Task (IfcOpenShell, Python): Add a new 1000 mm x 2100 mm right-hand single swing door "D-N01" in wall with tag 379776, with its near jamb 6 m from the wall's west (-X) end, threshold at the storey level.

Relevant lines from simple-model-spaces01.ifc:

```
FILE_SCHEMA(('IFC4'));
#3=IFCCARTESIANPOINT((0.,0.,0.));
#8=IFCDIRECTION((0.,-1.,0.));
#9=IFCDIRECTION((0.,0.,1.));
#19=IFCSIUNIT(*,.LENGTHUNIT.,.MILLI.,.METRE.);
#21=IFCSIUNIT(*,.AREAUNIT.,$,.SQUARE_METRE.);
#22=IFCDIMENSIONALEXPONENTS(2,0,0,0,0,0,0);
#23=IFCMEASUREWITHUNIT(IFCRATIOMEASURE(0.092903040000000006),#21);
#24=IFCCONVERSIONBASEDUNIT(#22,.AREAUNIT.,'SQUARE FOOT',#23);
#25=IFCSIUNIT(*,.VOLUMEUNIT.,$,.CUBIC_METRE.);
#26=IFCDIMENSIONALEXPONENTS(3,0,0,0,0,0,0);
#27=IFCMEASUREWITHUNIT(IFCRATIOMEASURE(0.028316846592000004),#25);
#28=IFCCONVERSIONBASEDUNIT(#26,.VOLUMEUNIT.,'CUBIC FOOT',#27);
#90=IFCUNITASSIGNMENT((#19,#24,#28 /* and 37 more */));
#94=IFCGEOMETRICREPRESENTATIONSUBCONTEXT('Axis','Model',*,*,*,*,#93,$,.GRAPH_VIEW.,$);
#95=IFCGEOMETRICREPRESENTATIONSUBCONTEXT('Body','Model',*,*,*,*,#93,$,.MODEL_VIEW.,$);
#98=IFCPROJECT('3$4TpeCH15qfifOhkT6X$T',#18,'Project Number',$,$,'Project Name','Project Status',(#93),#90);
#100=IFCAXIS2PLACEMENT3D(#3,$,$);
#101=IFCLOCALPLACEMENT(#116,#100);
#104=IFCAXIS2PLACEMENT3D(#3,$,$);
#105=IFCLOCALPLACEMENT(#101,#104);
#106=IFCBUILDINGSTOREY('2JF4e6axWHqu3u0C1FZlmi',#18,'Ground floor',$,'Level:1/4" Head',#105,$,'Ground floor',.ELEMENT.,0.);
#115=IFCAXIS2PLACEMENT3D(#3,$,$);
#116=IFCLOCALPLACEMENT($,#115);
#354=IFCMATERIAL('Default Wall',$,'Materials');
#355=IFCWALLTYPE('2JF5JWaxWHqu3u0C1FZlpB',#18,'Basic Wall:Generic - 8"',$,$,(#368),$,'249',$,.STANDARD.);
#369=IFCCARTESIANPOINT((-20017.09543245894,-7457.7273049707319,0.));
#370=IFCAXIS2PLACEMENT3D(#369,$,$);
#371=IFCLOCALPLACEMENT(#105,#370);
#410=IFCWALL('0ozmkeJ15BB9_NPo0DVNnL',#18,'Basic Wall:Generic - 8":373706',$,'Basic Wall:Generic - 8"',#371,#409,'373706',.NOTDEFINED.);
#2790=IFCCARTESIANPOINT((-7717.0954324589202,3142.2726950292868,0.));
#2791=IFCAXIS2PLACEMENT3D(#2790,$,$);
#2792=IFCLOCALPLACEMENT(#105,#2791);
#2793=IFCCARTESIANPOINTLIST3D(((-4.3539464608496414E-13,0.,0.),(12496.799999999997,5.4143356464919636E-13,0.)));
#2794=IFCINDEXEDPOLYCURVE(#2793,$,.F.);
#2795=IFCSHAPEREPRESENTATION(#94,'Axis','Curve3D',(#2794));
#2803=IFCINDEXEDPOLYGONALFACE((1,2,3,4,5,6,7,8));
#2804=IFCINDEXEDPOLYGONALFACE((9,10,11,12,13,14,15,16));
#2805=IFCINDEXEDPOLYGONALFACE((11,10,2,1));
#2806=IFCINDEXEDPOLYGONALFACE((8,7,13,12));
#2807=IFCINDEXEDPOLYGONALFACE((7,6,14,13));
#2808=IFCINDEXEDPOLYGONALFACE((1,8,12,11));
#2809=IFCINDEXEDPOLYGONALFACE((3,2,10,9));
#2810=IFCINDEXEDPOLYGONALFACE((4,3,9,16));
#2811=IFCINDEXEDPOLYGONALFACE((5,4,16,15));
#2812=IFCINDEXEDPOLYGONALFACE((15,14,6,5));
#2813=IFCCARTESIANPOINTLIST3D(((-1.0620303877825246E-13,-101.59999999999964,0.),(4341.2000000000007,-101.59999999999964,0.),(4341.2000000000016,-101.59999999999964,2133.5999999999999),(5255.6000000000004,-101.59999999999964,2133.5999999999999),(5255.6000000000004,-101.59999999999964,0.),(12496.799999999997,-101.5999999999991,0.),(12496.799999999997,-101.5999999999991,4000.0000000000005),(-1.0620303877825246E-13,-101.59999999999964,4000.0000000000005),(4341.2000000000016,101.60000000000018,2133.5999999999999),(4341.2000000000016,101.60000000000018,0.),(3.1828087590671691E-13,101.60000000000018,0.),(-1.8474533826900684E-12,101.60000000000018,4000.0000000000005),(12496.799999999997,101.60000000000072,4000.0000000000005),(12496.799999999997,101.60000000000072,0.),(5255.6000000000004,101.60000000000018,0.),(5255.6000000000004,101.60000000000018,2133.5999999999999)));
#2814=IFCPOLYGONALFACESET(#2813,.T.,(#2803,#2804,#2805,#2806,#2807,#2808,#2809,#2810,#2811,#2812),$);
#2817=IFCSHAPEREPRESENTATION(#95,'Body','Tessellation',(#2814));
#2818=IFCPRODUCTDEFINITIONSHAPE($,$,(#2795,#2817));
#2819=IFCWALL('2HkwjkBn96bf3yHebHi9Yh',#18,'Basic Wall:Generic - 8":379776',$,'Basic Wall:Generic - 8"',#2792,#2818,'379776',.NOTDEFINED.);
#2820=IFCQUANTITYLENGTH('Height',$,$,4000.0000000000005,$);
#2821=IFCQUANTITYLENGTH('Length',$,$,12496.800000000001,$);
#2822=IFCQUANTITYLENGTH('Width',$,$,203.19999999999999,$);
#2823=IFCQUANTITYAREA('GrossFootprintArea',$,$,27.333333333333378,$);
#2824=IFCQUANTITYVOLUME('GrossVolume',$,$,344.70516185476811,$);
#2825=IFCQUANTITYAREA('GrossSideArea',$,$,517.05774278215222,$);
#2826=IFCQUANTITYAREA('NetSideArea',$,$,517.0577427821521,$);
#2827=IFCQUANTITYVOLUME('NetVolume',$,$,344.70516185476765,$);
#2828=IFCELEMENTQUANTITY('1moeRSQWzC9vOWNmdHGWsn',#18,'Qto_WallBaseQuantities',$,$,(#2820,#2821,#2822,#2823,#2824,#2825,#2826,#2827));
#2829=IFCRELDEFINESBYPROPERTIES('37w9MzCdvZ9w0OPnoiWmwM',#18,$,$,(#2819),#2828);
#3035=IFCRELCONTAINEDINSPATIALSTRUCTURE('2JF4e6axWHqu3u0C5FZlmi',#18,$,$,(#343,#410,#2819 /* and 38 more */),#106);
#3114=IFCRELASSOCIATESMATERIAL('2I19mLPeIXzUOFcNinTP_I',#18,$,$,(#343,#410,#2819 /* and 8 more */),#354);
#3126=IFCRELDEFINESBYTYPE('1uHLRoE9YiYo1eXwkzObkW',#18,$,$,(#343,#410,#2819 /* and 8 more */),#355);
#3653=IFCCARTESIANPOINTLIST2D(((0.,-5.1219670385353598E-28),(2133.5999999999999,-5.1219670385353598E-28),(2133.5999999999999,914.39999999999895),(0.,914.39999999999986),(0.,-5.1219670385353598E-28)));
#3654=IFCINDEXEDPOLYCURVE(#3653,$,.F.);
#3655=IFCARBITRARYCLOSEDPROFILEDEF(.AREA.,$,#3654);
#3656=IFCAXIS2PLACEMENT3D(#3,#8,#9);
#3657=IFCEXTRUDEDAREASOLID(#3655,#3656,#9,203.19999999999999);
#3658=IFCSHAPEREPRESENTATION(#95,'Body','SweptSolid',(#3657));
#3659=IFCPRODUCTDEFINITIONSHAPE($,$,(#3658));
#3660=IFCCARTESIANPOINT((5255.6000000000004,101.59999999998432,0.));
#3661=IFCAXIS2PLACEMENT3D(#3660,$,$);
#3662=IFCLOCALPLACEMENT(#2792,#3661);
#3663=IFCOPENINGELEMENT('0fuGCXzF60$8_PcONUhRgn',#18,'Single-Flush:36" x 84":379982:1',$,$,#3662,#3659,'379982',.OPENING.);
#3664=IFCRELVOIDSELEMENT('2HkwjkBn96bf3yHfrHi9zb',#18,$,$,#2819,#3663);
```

```python
import numpy as np
import ifcopenshell
import ifcopenshell.api.feature
import ifcopenshell.api.geometry
import ifcopenshell.api.pset
import ifcopenshell.api.root
import ifcopenshell.api.spatial
import ifcopenshell.geom
import ifcopenshell.util.element
import ifcopenshell.util.placement
import ifcopenshell.util.representation
import ifcopenshell.util.shape
import ifcopenshell.util.unit

model = ifcopenshell.open("simple-model-spaces01.ifc")
unit_scale = ifcopenshell.util.unit.calculate_unit_scale(model)
area_scale = ifcopenshell.util.unit.calculate_unit_scale(model, "AREAUNIT")
volume_scale = ifcopenshell.util.unit.calculate_unit_scale(model, "VOLUMEUNIT")
settings = ifcopenshell.geom.settings()


def volume(element):
    """Net volume in cubic metres, openings subtracted."""
    shape = ifcopenshell.geom.create_shape(settings, element)
    return ifcopenshell.util.shape.get_volume(shape.geometry)


wall = model.by_guid("2HkwjkBn96bf3yHebHi9Yh")
storey = ifcopenshell.util.element.get_container(wall, ifc_class="IfcBuildingStorey")
context = ifcopenshell.util.representation.get_context(model, "Model", "Body", "MODEL_VIEW")
before = volume(wall)

width, height, from_end, sill = 1, 2.1, 6, 0.0  # metres

# The wall runs along its own X axis, and the end named is its -X end.
wall_shape = ifcopenshell.geom.create_shape(settings, wall)
x, y, z = ifcopenshell.util.shape.get_vertices(wall_shape.geometry).T
start = x.min() + from_end
face, thickness = float(y.min()), float(y.max() - y.min())
wall_matrix = ifcopenshell.util.placement.get_local_placement(wall.ObjectPlacement)
level = ifcopenshell.util.placement.get_local_placement(storey.ObjectPlacement)[2, 3]


def in_wall(x, y):
    """Placement at x, y metres in the wall's axes, at sill height."""
    matrix = wall_matrix.copy()
    matrix[:, 3] = wall_matrix @ np.array([x / unit_scale, y / unit_scale, 0.0, 1.0])
    matrix[2, 3] = level + sill / unit_scale
    return matrix


# Opening: a box that overshoots both wall faces by 50 mm.
opening = ifcopenshell.api.root.create_entity(model, ifc_class="IfcOpeningElement", predefined_type="OPENING")
box = ifcopenshell.api.geometry.add_wall_representation(
    model, context=context, length=width, height=height, thickness=thickness + 0.1
)
ifcopenshell.api.geometry.assign_representation(model, product=opening, representation=box)
ifcopenshell.api.geometry.edit_object_placement(model, product=opening, matrix=in_wall(start, face - 0.05), is_si=False)
ifcopenshell.api.feature.add_feature(model, feature=opening, element=wall)

door = ifcopenshell.api.root.create_entity(model, ifc_class="IfcDoor", name="D-N01", predefined_type="DOOR")
door.OverallWidth, door.OverallHeight = width / unit_scale, height / unit_scale
door.OperationType = "SINGLE_SWING_RIGHT"
body = ifcopenshell.api.geometry.add_door_representation(
    model,
    context=context,
    overall_width=door.OverallWidth,
    overall_height=door.OverallHeight,
    operation_type="SINGLE_SWING_RIGHT",
    lining_properties={"LiningDepth": thickness / unit_scale, "ThresholdDepth": thickness / unit_scale},
)
ifcopenshell.api.geometry.assign_representation(model, product=door, representation=body)
ifcopenshell.api.spatial.assign_container(model, products=[door], relating_structure=storey)
ifcopenshell.api.feature.add_filling(model, opening=opening, element=door)

# The lining spans the wall, so the door starts at the wall face.
ifcopenshell.api.geometry.edit_object_placement(model, product=door, matrix=in_wall(start, face), is_si=False)

after = volume(wall)

# Update the wall's stored quantities.
qto = model.by_id(ifcopenshell.util.element.get_pset(wall, "Qto_WallBaseQuantities", should_inherit=False)["id"])
ifcopenshell.api.pset.edit_qto(model, qto=qto, properties={
    "NetSideArea": after / thickness / area_scale,
    "NetVolume": after / volume_scale,
})

print(f"wall volume {before:.3f} -> {after:.3f} m3")

model.write("simple-model-spaces01_updated.ifc")
```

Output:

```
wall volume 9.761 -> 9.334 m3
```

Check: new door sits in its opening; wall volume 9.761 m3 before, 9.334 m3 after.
